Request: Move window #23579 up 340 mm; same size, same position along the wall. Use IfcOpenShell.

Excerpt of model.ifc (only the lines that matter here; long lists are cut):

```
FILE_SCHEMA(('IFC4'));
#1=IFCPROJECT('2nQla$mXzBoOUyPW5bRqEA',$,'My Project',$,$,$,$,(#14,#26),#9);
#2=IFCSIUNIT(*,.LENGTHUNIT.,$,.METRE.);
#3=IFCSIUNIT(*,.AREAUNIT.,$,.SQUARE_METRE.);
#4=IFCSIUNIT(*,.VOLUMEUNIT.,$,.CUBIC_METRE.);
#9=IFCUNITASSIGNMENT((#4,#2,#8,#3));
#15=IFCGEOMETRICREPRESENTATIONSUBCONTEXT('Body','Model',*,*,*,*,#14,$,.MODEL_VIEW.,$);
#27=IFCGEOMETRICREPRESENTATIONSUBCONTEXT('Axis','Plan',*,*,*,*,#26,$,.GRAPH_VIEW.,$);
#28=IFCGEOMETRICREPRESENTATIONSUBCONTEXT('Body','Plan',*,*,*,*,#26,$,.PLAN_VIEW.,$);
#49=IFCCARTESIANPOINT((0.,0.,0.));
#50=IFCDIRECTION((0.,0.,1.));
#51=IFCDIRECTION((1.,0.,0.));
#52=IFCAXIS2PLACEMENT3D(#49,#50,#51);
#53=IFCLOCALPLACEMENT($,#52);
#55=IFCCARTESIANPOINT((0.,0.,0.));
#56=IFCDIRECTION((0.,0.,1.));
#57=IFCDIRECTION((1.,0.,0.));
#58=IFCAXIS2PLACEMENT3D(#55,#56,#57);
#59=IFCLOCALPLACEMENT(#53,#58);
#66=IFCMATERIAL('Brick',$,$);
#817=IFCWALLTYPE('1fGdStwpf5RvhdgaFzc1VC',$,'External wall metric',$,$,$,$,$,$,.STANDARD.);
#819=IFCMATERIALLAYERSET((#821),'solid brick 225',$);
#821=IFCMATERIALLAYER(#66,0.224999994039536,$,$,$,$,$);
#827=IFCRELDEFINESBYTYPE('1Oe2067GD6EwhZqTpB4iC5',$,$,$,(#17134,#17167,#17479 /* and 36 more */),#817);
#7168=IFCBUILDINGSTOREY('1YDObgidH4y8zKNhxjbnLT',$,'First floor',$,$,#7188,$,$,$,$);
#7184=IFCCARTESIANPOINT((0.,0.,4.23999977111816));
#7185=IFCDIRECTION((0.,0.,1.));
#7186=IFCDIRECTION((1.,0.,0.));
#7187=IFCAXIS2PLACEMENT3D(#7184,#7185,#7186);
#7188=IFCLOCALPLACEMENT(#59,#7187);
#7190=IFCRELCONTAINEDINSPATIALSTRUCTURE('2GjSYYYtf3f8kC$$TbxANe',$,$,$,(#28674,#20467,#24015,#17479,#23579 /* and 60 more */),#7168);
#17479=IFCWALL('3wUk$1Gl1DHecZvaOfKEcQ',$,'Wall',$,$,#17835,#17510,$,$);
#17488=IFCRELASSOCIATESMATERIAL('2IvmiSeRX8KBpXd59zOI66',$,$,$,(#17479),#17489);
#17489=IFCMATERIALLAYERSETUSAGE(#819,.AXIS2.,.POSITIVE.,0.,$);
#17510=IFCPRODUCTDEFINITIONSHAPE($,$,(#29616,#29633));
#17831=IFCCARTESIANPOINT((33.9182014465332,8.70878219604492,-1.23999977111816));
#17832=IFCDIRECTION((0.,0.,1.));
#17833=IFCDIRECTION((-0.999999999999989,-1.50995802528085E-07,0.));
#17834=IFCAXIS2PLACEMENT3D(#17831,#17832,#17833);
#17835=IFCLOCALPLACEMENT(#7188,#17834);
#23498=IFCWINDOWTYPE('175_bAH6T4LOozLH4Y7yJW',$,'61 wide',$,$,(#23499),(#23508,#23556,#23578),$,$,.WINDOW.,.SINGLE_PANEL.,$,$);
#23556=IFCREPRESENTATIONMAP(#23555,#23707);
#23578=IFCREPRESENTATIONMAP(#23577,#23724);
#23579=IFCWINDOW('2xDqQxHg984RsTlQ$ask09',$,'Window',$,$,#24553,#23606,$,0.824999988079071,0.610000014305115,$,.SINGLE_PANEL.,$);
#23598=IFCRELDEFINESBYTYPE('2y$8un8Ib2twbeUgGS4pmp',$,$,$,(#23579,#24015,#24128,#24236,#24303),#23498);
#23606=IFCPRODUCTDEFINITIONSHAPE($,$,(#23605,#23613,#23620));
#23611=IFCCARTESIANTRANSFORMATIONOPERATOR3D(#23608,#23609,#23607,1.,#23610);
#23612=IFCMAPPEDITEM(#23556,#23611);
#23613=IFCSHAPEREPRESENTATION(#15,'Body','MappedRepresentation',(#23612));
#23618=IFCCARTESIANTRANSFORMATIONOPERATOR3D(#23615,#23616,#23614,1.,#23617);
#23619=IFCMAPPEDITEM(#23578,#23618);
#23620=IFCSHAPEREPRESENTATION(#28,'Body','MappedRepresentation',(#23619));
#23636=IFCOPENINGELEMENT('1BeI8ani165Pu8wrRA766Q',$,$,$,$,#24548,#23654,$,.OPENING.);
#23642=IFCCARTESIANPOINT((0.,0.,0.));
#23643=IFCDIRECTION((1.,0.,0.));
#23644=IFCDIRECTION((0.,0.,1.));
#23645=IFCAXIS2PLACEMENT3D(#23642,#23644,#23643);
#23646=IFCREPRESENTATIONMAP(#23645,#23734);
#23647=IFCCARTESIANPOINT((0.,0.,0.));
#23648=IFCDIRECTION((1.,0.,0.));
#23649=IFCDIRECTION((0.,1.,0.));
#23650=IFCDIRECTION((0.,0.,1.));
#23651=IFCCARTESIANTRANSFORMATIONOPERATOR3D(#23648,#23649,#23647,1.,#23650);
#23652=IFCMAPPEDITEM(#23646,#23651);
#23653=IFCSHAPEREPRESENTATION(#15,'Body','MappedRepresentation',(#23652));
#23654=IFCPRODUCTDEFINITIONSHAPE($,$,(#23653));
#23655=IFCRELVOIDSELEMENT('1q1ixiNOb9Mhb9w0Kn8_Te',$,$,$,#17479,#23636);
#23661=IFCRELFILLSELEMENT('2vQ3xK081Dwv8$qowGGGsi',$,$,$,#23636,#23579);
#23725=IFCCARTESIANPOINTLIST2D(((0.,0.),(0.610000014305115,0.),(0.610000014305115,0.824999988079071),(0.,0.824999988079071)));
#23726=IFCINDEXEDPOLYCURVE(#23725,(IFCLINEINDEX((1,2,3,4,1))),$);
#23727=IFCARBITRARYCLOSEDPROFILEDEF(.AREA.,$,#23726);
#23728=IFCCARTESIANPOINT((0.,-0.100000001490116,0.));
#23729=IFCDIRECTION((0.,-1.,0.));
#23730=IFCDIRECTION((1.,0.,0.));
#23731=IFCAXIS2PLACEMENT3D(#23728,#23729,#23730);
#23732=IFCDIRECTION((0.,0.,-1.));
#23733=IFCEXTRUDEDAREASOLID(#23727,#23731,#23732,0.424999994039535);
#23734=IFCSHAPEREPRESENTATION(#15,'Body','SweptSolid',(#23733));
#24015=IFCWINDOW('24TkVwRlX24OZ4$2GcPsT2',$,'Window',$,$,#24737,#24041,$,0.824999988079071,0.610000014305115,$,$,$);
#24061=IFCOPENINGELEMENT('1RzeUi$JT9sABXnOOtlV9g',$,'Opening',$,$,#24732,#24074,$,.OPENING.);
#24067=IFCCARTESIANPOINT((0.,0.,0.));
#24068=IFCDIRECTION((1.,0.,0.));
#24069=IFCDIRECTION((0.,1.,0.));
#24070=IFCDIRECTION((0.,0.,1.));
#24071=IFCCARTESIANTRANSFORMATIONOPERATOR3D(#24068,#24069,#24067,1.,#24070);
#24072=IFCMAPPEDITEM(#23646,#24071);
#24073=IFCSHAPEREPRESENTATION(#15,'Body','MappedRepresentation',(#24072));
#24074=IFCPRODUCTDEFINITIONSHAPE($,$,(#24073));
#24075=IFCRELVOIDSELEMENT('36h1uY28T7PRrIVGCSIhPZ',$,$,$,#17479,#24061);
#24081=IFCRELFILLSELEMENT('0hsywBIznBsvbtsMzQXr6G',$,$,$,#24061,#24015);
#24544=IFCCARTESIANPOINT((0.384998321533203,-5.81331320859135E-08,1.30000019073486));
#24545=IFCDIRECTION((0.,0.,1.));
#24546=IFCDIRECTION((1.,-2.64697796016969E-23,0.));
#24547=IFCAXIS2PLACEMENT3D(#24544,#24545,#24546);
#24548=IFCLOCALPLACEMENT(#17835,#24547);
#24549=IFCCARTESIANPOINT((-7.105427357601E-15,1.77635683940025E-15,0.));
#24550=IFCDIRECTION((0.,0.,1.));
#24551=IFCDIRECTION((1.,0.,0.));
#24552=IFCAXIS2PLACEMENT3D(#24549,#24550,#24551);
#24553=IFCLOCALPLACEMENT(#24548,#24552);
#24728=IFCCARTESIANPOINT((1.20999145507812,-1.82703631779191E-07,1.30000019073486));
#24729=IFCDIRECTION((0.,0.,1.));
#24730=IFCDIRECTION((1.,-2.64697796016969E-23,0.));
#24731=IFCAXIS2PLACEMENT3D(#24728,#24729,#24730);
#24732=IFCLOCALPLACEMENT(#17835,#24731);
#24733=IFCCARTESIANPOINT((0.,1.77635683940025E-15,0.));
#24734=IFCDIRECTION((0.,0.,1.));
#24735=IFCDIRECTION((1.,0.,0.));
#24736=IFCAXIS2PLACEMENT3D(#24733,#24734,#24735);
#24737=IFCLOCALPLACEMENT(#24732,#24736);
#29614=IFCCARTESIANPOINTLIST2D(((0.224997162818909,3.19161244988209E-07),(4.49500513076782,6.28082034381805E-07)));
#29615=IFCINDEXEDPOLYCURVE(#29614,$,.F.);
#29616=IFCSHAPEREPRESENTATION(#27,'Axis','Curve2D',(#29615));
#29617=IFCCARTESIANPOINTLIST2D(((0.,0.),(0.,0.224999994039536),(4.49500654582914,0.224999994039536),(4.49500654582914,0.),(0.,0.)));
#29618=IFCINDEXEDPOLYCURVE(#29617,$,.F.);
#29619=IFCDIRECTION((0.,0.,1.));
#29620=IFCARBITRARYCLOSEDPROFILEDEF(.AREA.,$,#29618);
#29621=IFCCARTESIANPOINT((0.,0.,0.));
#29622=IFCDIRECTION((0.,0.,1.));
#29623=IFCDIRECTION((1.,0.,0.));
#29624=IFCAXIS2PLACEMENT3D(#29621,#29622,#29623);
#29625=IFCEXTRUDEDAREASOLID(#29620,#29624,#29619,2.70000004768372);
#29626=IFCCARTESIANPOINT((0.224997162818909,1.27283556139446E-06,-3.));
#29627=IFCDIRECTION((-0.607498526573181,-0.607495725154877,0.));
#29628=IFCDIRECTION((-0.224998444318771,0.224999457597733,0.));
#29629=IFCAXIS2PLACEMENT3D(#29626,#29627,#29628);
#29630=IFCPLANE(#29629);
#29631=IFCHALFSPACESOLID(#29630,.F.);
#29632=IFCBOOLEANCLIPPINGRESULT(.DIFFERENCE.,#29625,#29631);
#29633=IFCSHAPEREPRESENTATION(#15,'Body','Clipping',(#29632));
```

```python
import numpy as np
import ifcopenshell
import ifcopenshell.api.geometry
import ifcopenshell.util.placement
import ifcopenshell.util.unit

model = ifcopenshell.open("model.ifc")
unit_scale = ifcopenshell.util.unit.calculate_unit_scale(model)

window = model.by_guid("2xDqQxHg984RsTlQ$ask09")
opening = window.FillsVoids[0].RelatingOpeningElement
dz = 0.34 / unit_scale

shift = np.array([0.0, 0.0, dz])
# The window is placed relative to its opening, so it follows when the opening moves.
matrix = ifcopenshell.util.placement.get_local_placement(opening.ObjectPlacement)
matrix[:3, 3] += shift
ifcopenshell.api.geometry.edit_object_placement(
    model, product=opening, matrix=matrix, is_si=False, should_transform_children=True
)

print(f"moved by {dz * unit_scale:+.3f} m")

model.write("model_edited.ifc")
```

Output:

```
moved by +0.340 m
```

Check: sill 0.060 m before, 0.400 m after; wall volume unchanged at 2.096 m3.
